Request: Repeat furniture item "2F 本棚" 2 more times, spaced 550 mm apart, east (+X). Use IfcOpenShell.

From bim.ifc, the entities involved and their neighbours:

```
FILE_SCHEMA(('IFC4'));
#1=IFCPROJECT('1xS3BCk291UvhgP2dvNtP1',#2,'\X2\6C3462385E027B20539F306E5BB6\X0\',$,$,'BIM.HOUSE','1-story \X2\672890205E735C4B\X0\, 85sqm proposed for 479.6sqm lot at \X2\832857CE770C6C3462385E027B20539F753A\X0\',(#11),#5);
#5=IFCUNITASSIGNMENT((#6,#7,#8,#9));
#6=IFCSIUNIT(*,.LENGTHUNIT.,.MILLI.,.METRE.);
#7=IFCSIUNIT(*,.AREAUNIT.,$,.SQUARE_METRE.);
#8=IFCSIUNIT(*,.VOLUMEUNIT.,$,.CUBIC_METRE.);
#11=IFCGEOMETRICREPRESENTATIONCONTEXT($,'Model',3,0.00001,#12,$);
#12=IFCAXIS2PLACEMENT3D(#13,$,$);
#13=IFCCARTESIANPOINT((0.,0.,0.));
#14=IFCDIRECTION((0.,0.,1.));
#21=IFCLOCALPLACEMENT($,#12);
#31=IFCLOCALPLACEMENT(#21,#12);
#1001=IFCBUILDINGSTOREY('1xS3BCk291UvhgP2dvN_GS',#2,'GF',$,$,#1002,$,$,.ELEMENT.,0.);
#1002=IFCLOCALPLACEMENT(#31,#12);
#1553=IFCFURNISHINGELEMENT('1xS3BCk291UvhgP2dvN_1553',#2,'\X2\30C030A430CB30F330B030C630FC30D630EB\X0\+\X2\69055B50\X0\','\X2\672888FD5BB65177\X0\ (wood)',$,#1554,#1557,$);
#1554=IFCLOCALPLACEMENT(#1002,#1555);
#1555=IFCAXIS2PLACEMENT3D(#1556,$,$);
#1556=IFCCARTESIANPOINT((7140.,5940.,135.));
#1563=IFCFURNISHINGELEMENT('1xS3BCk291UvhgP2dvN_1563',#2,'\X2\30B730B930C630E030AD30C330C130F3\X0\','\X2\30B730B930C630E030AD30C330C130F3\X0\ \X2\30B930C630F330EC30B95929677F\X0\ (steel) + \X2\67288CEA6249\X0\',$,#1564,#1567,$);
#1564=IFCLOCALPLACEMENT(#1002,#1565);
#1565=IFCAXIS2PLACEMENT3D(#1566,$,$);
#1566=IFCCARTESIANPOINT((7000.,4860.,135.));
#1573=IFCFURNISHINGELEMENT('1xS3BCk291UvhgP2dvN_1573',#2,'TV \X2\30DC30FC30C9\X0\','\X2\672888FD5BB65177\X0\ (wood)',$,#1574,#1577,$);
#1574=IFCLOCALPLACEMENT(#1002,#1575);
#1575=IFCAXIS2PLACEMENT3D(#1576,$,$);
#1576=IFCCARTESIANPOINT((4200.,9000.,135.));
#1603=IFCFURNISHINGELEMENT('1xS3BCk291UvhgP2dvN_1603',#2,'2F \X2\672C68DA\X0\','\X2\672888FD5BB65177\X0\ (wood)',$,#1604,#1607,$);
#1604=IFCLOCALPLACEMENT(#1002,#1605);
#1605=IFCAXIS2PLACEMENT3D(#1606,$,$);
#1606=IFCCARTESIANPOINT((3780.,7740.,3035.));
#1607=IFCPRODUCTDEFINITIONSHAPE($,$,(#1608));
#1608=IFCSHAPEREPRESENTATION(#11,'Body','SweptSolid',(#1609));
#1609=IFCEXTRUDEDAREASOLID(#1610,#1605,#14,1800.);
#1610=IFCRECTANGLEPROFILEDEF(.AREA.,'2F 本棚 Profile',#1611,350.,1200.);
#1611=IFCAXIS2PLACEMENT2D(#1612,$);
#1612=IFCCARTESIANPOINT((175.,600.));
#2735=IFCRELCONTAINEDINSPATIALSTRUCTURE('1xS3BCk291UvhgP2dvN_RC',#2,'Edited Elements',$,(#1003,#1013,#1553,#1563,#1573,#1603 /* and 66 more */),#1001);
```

```python
import numpy as np
import ifcopenshell
import ifcopenshell.api.geometry
import ifcopenshell.api.root
import ifcopenshell.util.element
import ifcopenshell.util.placement

model = ifcopenshell.open("bim.ifc")


def reuse_history(source, copy):
    """copy_class also copies each property set's owner history, people and application; keep the originals."""
    for rel in copy.IsDefinedBy:
        if rel.is_a("IfcRelDefinesByProperties") and (history := rel.RelatingPropertyDefinition.OwnerHistory):
            rel.RelatingPropertyDefinition.OwnerHistory = source.OwnerHistory
            ifcopenshell.util.element.remove_deep2(model, history)


source = model.by_guid("1xS3BCk291UvhgP2dvN_1603")
base = ifcopenshell.util.placement.get_local_placement(source.ObjectPlacement)
step = np.array([1.0, 0.0, 0.0]) * 550.0

for i in range(1, 3):
    copy = ifcopenshell.api.root.copy_class(model, product=source)
    copy.Representation = ifcopenshell.util.element.copy_deep(
        model, source.Representation, exclude=["IfcGeometricRepresentationContext", "IfcRepresentationMap"]
    )
    reuse_history(source, copy)
    matrix = base.copy()
    matrix[:3, 3] += i * step
    print("added at", matrix[:3, 3].round(3) + 0.0)
    ifcopenshell.api.geometry.edit_object_placement(model, product=copy, matrix=matrix, is_si=False)

model.write("bim_rev.ifc")
```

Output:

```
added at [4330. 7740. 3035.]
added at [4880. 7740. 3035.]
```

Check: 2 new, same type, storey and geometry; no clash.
